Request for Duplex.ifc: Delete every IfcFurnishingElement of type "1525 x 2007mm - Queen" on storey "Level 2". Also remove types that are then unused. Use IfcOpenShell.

First a look at what the model holds.

```python
import ifcopenshell
import ifcopenshell.util.element

model = ifcopenshell.open("Duplex.ifc")
print(model.schema)
storey = next(s for s in model.by_type("IfcBuildingStorey") if s.Name == "Level 2")
furniture = [e for e in ifcopenshell.util.element.get_decomposition(storey) if e.is_a("IfcFurnishingElement")]
seen = {}
for e in furniture:
    element_type = ifcopenshell.util.element.get_type(e)
    name = element_type.Name if element_type not in (None, e) else None
    seen[name] = seen.get(name, 0) + 1
for name, count in sorted(seen.items(), key=str):
    print(count, "x", name)
```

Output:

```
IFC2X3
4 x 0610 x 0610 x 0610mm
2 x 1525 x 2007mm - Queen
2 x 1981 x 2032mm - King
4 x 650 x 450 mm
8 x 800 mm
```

```python
import ifcopenshell
import ifcopenshell.api.root
import ifcopenshell.util.element

model = ifcopenshell.open("Duplex.ifc")

storey = next(s for s in model.by_type("IfcBuildingStorey") if s.Name == "Level 2")
furniture = [e for e in ifcopenshell.util.element.get_decomposition(storey) if e.is_a("IfcFurnishingElement")]
targets = [e for e in furniture if (t := ifcopenshell.util.element.get_type(e)) not in (None, e) and t.Name == "1525 x 2007mm - Queen"]
types = {ifcopenshell.util.element.get_type(e) for e in targets} - {None, *targets}

for e in targets:
    ifcopenshell.api.root.remove_product(model, product=e)
print(len(targets), "removed")

unused = [t for t in types if not ifcopenshell.util.element.get_types(t)]
for t in unused:
    ifcopenshell.api.root.remove_product(model, product=t)
print(len(unused), "unused types removed")

model.write("Duplex-out.ifc")
```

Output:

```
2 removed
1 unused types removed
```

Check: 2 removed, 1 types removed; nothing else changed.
